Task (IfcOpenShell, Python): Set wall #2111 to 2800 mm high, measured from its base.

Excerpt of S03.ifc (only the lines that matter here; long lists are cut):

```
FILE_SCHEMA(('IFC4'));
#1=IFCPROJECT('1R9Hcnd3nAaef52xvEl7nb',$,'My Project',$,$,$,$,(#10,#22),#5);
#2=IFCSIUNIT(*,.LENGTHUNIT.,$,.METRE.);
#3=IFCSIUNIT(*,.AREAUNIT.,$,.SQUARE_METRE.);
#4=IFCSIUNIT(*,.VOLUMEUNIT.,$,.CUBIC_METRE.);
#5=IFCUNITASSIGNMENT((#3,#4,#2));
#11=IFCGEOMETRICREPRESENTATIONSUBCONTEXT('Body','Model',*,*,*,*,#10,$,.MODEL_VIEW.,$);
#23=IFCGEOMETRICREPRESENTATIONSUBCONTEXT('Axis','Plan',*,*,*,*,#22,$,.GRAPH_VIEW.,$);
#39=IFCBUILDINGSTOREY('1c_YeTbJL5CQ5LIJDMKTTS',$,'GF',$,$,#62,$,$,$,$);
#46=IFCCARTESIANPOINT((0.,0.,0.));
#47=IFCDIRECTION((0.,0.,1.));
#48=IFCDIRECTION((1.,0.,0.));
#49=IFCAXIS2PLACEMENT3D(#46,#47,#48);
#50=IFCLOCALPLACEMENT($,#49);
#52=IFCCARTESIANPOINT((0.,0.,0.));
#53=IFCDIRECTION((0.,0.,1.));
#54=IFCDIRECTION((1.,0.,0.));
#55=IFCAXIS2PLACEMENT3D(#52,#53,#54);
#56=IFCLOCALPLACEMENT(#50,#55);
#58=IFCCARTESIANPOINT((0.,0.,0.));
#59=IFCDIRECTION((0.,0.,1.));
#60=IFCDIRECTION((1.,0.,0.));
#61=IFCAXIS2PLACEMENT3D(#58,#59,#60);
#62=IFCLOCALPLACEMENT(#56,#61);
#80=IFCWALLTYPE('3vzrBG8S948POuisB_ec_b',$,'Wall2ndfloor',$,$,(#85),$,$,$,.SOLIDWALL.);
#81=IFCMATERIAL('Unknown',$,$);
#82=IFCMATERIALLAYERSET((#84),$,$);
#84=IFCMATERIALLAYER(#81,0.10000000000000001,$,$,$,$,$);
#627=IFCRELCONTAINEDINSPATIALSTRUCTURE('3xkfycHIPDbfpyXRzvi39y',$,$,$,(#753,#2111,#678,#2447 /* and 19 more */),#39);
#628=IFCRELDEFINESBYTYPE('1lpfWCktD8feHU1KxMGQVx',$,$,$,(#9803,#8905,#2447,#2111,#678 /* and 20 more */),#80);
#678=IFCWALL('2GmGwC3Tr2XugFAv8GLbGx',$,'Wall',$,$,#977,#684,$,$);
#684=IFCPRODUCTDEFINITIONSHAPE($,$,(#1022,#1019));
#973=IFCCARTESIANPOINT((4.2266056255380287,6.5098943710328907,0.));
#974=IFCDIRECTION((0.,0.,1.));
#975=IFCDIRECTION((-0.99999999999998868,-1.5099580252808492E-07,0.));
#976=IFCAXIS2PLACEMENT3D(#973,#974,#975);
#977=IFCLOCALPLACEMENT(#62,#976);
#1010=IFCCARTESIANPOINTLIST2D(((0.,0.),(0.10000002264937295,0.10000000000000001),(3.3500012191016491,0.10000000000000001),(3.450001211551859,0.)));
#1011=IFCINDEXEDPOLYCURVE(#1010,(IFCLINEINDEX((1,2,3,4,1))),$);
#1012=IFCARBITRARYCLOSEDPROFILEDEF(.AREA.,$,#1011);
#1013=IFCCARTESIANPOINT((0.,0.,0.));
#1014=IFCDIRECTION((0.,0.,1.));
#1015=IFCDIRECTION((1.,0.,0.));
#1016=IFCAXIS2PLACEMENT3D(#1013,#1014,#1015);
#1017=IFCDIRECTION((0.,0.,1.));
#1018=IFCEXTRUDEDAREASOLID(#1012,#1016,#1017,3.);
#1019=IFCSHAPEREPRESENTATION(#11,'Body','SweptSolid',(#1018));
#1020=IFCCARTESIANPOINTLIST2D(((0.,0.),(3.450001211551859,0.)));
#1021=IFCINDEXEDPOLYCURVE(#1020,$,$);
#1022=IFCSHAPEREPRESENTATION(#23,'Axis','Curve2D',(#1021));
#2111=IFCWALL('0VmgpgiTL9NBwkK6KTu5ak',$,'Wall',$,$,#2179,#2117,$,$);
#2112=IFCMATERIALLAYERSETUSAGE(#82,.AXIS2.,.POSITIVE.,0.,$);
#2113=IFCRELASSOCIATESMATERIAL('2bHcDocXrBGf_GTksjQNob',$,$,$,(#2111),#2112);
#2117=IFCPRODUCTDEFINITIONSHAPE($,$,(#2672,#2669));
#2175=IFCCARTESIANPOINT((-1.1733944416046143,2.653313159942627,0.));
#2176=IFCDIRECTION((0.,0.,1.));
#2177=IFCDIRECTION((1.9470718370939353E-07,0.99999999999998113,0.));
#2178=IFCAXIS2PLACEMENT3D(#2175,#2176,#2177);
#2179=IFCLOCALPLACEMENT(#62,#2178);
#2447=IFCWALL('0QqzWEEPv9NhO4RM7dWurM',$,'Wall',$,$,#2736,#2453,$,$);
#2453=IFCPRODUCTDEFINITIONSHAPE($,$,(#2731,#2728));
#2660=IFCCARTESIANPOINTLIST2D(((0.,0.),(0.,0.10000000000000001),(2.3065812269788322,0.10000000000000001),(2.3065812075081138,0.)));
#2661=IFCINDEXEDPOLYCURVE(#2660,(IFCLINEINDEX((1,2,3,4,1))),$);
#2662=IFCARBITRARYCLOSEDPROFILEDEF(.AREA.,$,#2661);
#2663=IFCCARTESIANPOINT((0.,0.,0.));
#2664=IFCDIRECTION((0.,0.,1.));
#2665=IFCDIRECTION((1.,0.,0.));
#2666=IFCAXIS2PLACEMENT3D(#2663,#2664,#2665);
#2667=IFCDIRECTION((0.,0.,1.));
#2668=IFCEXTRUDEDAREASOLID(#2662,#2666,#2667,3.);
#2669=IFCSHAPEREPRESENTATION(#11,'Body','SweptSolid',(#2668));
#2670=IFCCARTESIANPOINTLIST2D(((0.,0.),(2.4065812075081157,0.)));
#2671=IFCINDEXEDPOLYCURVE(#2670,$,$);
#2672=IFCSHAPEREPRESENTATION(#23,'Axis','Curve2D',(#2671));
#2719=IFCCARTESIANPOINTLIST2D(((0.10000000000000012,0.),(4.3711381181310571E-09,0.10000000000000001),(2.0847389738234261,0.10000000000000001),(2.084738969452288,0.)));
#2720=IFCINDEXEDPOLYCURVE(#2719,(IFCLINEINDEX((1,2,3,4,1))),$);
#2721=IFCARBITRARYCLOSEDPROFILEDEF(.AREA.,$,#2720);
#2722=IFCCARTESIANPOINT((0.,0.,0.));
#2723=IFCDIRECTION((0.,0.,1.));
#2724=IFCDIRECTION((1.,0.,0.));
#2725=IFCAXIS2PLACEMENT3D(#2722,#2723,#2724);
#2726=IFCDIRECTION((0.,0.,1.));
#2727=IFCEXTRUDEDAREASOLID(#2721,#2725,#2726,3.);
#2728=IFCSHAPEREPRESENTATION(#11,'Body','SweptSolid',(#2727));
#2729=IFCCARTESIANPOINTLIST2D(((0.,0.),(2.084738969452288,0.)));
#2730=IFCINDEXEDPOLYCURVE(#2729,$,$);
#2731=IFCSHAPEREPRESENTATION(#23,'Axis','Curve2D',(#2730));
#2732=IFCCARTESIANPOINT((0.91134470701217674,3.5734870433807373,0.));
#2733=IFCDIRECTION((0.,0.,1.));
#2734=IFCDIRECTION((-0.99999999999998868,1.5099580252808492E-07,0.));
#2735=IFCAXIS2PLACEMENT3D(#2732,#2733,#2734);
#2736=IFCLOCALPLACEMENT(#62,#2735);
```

```python
import ifcopenshell
import ifcopenshell.geom
import ifcopenshell.util.representation
import ifcopenshell.util.shape
import ifcopenshell.util.unit

model = ifcopenshell.open("S03.ifc")
unit_scale = ifcopenshell.util.unit.calculate_unit_scale(model)
settings = ifcopenshell.geom.settings()


def volume(element):
    """Net volume in cubic metres, openings subtracted."""
    shape = ifcopenshell.geom.create_shape(settings, element)
    return ifcopenshell.util.shape.get_volume(shape.geometry)


wall = model.by_guid("0VmgpgiTL9NBwkK6KTu5ak")
before = volume(wall)

body = ifcopenshell.util.representation.get_representation(wall, "Model", "Body")
solid = body.Items[0]
old_height = solid.Depth
solid.Depth = 2.8 / unit_scale
after = volume(wall)

print(f"height {old_height:g} -> {solid.Depth:g}, volume {before:.3f} -> {after:.3f} m3")

model.write("S03_v2.ifc")
```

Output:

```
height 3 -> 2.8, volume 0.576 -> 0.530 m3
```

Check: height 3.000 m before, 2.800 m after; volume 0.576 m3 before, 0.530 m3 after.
